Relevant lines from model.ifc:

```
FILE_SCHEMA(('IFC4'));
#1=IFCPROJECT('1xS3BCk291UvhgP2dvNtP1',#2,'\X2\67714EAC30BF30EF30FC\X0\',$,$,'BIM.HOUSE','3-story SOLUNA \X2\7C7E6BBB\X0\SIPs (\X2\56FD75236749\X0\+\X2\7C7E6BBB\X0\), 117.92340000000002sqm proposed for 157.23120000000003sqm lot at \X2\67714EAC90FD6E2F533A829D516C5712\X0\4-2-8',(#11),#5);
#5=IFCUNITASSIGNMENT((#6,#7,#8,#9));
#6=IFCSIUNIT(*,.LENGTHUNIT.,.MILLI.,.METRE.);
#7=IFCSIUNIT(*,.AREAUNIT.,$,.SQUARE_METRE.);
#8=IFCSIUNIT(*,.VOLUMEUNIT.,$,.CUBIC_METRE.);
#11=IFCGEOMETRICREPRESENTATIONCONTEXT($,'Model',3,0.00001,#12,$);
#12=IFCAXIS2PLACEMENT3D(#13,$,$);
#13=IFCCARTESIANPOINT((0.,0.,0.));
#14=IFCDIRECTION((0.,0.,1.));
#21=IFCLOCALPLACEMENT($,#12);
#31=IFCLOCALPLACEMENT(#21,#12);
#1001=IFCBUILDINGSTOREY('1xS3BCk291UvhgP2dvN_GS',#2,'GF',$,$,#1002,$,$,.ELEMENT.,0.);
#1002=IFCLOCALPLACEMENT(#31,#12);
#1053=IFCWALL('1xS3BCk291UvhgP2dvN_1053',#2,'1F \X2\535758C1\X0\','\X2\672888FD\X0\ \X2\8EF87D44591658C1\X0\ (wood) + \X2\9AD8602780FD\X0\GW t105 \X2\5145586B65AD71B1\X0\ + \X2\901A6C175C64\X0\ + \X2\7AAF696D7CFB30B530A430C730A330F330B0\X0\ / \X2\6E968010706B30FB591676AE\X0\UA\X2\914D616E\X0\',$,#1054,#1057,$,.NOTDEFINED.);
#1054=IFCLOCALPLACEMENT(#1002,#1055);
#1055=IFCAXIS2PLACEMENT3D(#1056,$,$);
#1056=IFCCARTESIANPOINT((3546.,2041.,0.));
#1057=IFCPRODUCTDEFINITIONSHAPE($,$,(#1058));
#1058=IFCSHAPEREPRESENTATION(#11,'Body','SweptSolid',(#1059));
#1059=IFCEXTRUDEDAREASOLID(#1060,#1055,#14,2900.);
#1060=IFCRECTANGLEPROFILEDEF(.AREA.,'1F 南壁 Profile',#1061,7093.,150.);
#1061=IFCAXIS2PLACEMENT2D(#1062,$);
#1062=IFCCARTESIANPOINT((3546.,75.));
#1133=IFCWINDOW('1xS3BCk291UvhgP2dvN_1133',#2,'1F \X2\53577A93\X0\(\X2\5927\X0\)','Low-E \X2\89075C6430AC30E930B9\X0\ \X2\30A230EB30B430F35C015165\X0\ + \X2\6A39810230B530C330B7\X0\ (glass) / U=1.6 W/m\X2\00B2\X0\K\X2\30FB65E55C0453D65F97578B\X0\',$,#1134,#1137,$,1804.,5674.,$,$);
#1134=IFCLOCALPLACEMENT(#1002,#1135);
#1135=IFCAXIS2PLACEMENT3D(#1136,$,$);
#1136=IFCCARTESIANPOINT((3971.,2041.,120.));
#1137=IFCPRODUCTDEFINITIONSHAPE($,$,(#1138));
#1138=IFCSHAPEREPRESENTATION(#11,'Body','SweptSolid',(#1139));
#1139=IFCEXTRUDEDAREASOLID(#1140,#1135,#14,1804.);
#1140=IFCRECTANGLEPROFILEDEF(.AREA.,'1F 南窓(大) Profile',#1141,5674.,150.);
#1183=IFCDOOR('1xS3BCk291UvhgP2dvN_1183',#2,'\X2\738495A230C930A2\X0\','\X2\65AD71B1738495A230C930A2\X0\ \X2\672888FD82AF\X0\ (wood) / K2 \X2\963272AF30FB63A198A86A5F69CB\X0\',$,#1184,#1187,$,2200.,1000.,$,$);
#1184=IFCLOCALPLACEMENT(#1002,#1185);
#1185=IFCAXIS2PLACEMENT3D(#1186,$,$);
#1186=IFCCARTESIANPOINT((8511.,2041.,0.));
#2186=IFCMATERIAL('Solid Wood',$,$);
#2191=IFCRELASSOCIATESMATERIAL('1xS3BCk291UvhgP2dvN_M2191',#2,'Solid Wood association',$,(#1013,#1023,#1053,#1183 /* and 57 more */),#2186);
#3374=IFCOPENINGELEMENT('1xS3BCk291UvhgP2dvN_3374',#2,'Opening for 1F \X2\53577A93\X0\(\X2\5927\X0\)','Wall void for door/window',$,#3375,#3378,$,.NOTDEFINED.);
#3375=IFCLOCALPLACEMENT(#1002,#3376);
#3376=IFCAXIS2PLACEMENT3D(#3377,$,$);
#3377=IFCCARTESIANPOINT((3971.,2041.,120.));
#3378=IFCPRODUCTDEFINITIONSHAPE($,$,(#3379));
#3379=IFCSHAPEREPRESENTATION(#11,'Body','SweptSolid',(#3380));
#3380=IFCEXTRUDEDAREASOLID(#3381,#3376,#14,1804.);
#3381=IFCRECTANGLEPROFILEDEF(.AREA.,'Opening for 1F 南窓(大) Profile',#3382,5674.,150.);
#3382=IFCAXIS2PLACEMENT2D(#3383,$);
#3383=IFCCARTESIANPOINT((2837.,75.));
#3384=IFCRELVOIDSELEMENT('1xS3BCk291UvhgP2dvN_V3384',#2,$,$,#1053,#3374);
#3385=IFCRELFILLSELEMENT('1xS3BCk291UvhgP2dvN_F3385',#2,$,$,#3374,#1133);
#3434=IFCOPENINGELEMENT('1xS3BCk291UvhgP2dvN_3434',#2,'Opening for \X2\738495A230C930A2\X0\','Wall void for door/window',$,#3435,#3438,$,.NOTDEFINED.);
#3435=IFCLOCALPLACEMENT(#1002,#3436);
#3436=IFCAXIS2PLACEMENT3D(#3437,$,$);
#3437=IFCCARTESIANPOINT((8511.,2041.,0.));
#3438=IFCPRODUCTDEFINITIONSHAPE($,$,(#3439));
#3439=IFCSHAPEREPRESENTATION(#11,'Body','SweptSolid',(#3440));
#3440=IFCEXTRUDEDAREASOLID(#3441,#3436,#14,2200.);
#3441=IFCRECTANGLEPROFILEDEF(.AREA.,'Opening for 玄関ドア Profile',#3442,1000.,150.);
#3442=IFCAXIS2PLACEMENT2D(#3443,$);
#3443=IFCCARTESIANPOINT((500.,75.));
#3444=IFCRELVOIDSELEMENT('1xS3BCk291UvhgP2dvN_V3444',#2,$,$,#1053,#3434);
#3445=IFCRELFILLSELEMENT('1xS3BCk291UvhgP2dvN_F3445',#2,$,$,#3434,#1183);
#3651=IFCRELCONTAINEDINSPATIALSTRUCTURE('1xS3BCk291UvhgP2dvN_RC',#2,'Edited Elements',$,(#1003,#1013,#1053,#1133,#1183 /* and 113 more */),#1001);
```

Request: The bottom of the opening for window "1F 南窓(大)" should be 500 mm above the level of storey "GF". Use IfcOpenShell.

```python
import numpy as np
import ifcopenshell
import ifcopenshell.api.geometry
import ifcopenshell.geom
import ifcopenshell.util.element
import ifcopenshell.util.placement
import ifcopenshell.util.shape
import ifcopenshell.util.unit

model = ifcopenshell.open("model.ifc")
unit_scale = ifcopenshell.util.unit.calculate_unit_scale(model)

window = model.by_id(1133)
opening = window.FillsVoids[0].RelatingOpeningElement
storey = ifcopenshell.util.element.get_container(window, ifc_class="IfcBuildingStorey")
level = ifcopenshell.util.placement.get_local_placement(storey.ObjectPlacement)[2, 3]

# The opening's origin need not be at the sill, so measure its lowest point.
shape = ifcopenshell.geom.create_shape(ifcopenshell.geom.settings(), opening)
bottom = ifcopenshell.util.shape.get_shape_bottom_elevation(shape, shape.geometry) / unit_scale
dz = level + 500.0 - bottom

shift = np.array([0.0, 0.0, dz])
# The window is not placed relative to its opening, so move both.
for product in (opening, window):
    matrix = ifcopenshell.util.placement.get_local_placement(product.ObjectPlacement)
    matrix[:3, 3] += shift
    ifcopenshell.api.geometry.edit_object_placement(model, product=product, matrix=matrix, is_si=False)

print(f"moved by {dz * unit_scale:+.3f} m")

model.write("model_updated.ifc")
```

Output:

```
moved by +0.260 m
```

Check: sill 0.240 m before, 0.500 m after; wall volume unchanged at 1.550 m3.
